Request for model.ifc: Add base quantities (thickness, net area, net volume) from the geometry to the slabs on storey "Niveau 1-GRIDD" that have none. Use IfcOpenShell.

First a look at what the model holds.

```python
import ifcopenshell
import ifcopenshell.util.element
import ifcopenshell.util.unit

model = ifcopenshell.open("model.ifc")
print(model.schema)
for unit_type in ("LENGTHUNIT", "AREAUNIT", "VOLUMEUNIT"):
    print(unit_type, ifcopenshell.util.unit.calculate_unit_scale(model, unit_type))
storey = next(s for s in model.by_type("IfcBuildingStorey") if s.Name == "Niveau 1-GRIDD")
slabs = [e for e in ifcopenshell.util.element.get_decomposition(storey) if e.is_a("IfcSlab")]
for e in sorted(slabs, key=lambda e: e.id()):
    print(e.id(), e.is_a(), e.Name, list(ifcopenshell.util.element.get_psets(e, qtos_only=True)), sep=" | ")
```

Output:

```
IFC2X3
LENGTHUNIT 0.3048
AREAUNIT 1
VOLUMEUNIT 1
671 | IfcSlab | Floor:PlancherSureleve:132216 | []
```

```python
import ifcopenshell
import ifcopenshell.api.pset
import ifcopenshell.geom
import ifcopenshell.util.element
import ifcopenshell.util.shape
import ifcopenshell.util.unit

model = ifcopenshell.open("model.ifc")
unit_scale = ifcopenshell.util.unit.calculate_unit_scale(model)
area_scale = ifcopenshell.util.unit.calculate_unit_scale(model, "AREAUNIT")
volume_scale = ifcopenshell.util.unit.calculate_unit_scale(model, "VOLUMEUNIT")
settings = ifcopenshell.geom.settings()

storey = next(s for s in model.by_type("IfcBuildingStorey") if s.Name == "Niveau 1-GRIDD")
slabs = [e for e in ifcopenshell.util.element.get_decomposition(storey) if e.is_a("IfcSlab")]

for e in sorted(slabs, key=lambda e: e.id()):
    if ifcopenshell.util.element.get_psets(e, qtos_only=True, should_inherit=False):
        continue
    # Geometry comes back in metres, in the element's own axes.
    shape = ifcopenshell.geom.create_shape(settings, e)
    values = {
        "Width": ifcopenshell.util.shape.get_z(shape.geometry) / unit_scale,
        "NetArea": ifcopenshell.util.shape.get_footprint_area(shape.geometry) / area_scale,
        "NetVolume": ifcopenshell.util.shape.get_volume(shape.geometry) / volume_scale,
    }
    qto = ifcopenshell.api.pset.add_qto(model, product=e, name="BaseQuantities")
    ifcopenshell.api.pset.edit_qto(model, qto=qto, properties=values)
    print(e.id(), {k: round(v, 3) for k, v in values.items()})

model.write("model_updated.ifc")
```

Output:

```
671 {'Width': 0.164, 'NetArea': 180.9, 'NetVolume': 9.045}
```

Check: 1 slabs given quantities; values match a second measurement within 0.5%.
